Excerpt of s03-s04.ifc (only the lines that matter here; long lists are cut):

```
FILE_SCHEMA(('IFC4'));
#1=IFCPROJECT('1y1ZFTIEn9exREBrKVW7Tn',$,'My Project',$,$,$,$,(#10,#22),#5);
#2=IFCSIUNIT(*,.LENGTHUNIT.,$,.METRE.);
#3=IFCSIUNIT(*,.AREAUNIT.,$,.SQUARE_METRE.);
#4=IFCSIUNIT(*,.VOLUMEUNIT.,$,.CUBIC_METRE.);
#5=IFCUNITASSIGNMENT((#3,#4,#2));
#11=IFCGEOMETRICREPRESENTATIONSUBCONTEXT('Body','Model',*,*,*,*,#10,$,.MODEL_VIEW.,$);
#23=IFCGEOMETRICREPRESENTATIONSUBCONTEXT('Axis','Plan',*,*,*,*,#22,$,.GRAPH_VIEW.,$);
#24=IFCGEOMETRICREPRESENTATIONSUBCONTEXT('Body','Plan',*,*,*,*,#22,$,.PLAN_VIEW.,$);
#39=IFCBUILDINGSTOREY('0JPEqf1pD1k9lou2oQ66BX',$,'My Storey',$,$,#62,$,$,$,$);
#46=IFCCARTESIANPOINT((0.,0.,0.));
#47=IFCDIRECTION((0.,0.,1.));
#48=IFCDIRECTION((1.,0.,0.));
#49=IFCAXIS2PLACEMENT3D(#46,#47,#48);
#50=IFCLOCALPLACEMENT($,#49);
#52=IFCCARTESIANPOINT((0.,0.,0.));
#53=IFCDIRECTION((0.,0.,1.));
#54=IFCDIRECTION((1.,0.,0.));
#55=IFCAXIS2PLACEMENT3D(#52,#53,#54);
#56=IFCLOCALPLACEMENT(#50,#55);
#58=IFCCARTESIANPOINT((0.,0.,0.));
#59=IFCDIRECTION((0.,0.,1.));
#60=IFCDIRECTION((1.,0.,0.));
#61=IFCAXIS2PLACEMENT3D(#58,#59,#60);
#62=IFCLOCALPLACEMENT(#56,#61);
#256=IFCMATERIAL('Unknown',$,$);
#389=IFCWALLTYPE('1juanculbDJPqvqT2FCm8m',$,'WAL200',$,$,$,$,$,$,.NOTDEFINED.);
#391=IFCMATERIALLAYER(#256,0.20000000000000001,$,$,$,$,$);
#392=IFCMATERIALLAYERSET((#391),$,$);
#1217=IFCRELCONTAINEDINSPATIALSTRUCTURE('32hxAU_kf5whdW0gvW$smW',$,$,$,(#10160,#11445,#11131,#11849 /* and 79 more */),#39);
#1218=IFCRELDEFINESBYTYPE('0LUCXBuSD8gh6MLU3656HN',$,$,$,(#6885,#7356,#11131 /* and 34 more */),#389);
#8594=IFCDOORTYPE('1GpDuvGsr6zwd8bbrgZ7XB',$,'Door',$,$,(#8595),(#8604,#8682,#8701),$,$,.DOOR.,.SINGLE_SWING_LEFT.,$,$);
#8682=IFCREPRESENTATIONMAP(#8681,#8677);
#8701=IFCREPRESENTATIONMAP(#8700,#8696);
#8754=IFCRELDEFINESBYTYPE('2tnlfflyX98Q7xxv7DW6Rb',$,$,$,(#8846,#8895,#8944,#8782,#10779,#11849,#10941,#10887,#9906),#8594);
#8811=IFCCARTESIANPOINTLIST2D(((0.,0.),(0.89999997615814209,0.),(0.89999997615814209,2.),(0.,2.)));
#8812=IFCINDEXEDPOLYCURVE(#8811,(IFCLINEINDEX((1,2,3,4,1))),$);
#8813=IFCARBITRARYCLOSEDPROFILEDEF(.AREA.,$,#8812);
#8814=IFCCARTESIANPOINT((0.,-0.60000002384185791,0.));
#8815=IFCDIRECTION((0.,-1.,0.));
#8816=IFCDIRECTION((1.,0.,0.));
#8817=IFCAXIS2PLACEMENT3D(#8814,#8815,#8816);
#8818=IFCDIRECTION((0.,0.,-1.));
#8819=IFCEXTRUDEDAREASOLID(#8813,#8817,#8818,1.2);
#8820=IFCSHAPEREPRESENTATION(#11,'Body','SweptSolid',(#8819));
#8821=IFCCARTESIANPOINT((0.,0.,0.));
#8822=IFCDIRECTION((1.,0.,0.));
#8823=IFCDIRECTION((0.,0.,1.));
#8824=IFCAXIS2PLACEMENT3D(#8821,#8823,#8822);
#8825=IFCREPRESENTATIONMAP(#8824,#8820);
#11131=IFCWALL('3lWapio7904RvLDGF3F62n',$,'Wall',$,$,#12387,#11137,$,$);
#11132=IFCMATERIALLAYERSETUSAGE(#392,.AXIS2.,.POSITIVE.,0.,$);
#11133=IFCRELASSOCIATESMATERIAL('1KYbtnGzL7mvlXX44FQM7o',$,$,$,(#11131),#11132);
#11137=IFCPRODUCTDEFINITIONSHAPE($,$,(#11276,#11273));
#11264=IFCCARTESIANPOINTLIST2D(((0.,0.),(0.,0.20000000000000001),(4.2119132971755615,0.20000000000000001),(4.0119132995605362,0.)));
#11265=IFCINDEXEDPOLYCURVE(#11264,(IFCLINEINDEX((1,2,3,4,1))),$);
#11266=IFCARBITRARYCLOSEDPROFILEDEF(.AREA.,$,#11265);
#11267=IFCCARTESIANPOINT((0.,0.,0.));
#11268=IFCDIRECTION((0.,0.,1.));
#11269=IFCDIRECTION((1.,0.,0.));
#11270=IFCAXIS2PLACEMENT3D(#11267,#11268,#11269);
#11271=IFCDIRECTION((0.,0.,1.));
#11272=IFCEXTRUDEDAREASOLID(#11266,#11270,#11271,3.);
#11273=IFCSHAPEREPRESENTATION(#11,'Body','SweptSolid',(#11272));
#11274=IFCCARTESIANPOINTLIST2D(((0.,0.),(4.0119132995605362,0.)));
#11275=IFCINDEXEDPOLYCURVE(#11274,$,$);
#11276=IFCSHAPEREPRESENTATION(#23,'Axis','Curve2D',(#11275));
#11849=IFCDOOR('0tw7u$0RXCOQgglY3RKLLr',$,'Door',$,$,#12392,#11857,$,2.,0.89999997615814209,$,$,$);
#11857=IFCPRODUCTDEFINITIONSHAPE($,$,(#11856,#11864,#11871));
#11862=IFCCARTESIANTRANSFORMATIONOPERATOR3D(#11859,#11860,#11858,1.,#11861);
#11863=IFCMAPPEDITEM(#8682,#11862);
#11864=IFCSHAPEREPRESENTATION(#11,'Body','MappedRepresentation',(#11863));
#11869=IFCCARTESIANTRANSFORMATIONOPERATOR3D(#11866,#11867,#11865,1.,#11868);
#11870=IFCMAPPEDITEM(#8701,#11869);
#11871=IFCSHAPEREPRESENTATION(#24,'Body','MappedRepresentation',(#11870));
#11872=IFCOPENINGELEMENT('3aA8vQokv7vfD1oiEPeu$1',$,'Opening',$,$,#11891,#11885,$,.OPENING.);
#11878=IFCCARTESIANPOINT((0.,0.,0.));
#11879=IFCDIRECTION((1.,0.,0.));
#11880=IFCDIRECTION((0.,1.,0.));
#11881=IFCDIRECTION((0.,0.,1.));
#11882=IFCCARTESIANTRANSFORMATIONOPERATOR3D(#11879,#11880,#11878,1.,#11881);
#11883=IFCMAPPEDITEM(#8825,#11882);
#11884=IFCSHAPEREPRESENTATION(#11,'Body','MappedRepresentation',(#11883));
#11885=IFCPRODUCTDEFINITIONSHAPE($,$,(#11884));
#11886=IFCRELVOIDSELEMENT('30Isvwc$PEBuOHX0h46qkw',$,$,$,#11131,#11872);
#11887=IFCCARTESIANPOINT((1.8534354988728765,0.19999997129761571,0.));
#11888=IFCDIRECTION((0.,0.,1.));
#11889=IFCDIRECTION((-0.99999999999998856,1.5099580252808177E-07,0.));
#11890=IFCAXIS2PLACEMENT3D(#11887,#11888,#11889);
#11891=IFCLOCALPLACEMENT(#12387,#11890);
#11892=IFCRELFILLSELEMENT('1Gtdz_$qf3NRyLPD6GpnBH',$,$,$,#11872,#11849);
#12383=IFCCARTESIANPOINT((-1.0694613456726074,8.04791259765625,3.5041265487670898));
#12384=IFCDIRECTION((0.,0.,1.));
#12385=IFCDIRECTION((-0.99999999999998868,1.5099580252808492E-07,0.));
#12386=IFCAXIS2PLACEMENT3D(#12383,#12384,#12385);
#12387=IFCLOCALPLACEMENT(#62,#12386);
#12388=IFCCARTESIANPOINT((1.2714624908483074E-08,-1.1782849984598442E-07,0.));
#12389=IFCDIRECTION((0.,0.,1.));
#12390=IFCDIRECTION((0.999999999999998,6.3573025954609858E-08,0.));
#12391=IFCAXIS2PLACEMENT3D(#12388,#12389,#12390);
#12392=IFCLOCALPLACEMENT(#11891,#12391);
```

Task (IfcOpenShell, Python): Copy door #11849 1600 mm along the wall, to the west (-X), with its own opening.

```python
import ifcopenshell
import ifcopenshell.api.feature
import ifcopenshell.api.geometry
import ifcopenshell.api.root
import ifcopenshell.geom
import ifcopenshell.util.element
import ifcopenshell.util.placement
import ifcopenshell.util.shape
import ifcopenshell.util.unit

model = ifcopenshell.open("s03-s04.ifc")
unit_scale = ifcopenshell.util.unit.calculate_unit_scale(model)
settings = ifcopenshell.geom.settings()


def volume(element):
    """Net volume in cubic metres, openings subtracted."""
    shape = ifcopenshell.geom.create_shape(settings, element)
    return ifcopenshell.util.shape.get_volume(shape.geometry)


door = model.by_id(11849)
opening = door.FillsVoids[0].RelatingOpeningElement
wall = opening.VoidsElements[0].RelatingBuildingElement
before = volume(wall)
shift = ifcopenshell.util.placement.get_local_placement(wall.ObjectPlacement)[:3, 0] * 1.6 / unit_scale

# copy_class copies the void relationship, type, container and properties, but no geometry.
new_opening = ifcopenshell.api.root.copy_class(model, product=opening)
new_opening.Representation = ifcopenshell.util.element.copy_deep(
    model, opening.Representation, exclude=["IfcGeometricRepresentationContext", "IfcRepresentationMap"]
)
new_door = ifcopenshell.api.root.copy_class(model, product=door)
new_door.Representation = ifcopenshell.util.element.copy_deep(
    model, door.Representation, exclude=["IfcGeometricRepresentationContext", "IfcRepresentationMap"]
)
ifcopenshell.api.feature.add_filling(model, opening=new_opening, element=new_door)

for old, new in ((opening, new_opening), (door, new_door)):
    matrix = ifcopenshell.util.placement.get_local_placement(old.ObjectPlacement)
    matrix[:3, 3] += shift
    ifcopenshell.api.geometry.edit_object_placement(model, product=new, matrix=matrix, is_si=False)

after = volume(wall)

print(f"wall volume {before:.3f} -> {after:.3f} m3")

model.write("s03-s04-out.ifc")
```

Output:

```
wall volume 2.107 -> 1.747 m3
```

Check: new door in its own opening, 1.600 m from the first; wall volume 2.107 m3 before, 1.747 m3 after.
